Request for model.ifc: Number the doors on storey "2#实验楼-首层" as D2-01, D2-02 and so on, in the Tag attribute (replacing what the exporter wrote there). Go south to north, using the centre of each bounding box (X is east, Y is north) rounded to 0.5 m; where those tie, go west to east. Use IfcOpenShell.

First a look at what the model holds.

```python
import ifcopenshell
import ifcopenshell.util.element
import ifcopenshell.util.placement

model = ifcopenshell.open("model.ifc")
print(model.schema)
storey = next(s for s in model.by_type("IfcBuildingStorey") if s.Name == "2#实验楼-首层")
doors = [e for e in ifcopenshell.util.element.get_decomposition(storey) if e.is_a("IfcDoor")]
for e in sorted(doors, key=lambda e: e.id()):
    origin = ifcopenshell.util.placement.get_local_placement(e.ObjectPlacement)[:3, 3]
    print(e.id(), e.Tag, e.Name, origin.round(2) + 0.0, sep=" | ")
```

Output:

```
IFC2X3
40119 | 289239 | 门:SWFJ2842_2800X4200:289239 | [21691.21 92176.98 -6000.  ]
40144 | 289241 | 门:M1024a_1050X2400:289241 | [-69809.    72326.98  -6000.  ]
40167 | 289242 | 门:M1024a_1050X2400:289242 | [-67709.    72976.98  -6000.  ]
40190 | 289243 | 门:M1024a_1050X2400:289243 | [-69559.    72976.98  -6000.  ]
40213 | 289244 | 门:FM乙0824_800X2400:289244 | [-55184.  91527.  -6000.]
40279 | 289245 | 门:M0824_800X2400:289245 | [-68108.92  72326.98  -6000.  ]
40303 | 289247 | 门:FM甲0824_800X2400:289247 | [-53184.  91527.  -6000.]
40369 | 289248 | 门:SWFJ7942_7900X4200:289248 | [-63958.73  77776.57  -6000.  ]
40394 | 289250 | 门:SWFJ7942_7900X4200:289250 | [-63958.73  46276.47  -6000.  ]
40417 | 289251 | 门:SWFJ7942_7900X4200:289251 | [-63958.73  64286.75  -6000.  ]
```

```python
import ifcopenshell
import ifcopenshell.geom
import ifcopenshell.util.element
import ifcopenshell.util.shape

model = ifcopenshell.open("model.ifc")
settings = ifcopenshell.geom.settings()
settings.set("use-world-coords", True)


def centre(element):
    shape = ifcopenshell.geom.create_shape(settings, element)
    return ifcopenshell.util.shape.get_bbox_centroid(shape.geometry)


storey = next(s for s in model.by_type("IfcBuildingStorey") if s.Name == "2#实验楼-首层")
doors = [e for e in ifcopenshell.util.element.get_decomposition(storey) if e.is_a("IfcDoor")]

# Insertion points can sit at a corner or the storey origin, so sort by the geometry (in metres).
centres = {e: centre(e) for e in doors}
doors.sort(key=lambda e: (round(centres[e][1] / 0.5), centres[e][0]))

for i, e in enumerate(doors, start=1):
    number = f"D2-{i:02d}"
    e.Tag = number
    print(e.id(), number)

model.write("model-out.ifc")
```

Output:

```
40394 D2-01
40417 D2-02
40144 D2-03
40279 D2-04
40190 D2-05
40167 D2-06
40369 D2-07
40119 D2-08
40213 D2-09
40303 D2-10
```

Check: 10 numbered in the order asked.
